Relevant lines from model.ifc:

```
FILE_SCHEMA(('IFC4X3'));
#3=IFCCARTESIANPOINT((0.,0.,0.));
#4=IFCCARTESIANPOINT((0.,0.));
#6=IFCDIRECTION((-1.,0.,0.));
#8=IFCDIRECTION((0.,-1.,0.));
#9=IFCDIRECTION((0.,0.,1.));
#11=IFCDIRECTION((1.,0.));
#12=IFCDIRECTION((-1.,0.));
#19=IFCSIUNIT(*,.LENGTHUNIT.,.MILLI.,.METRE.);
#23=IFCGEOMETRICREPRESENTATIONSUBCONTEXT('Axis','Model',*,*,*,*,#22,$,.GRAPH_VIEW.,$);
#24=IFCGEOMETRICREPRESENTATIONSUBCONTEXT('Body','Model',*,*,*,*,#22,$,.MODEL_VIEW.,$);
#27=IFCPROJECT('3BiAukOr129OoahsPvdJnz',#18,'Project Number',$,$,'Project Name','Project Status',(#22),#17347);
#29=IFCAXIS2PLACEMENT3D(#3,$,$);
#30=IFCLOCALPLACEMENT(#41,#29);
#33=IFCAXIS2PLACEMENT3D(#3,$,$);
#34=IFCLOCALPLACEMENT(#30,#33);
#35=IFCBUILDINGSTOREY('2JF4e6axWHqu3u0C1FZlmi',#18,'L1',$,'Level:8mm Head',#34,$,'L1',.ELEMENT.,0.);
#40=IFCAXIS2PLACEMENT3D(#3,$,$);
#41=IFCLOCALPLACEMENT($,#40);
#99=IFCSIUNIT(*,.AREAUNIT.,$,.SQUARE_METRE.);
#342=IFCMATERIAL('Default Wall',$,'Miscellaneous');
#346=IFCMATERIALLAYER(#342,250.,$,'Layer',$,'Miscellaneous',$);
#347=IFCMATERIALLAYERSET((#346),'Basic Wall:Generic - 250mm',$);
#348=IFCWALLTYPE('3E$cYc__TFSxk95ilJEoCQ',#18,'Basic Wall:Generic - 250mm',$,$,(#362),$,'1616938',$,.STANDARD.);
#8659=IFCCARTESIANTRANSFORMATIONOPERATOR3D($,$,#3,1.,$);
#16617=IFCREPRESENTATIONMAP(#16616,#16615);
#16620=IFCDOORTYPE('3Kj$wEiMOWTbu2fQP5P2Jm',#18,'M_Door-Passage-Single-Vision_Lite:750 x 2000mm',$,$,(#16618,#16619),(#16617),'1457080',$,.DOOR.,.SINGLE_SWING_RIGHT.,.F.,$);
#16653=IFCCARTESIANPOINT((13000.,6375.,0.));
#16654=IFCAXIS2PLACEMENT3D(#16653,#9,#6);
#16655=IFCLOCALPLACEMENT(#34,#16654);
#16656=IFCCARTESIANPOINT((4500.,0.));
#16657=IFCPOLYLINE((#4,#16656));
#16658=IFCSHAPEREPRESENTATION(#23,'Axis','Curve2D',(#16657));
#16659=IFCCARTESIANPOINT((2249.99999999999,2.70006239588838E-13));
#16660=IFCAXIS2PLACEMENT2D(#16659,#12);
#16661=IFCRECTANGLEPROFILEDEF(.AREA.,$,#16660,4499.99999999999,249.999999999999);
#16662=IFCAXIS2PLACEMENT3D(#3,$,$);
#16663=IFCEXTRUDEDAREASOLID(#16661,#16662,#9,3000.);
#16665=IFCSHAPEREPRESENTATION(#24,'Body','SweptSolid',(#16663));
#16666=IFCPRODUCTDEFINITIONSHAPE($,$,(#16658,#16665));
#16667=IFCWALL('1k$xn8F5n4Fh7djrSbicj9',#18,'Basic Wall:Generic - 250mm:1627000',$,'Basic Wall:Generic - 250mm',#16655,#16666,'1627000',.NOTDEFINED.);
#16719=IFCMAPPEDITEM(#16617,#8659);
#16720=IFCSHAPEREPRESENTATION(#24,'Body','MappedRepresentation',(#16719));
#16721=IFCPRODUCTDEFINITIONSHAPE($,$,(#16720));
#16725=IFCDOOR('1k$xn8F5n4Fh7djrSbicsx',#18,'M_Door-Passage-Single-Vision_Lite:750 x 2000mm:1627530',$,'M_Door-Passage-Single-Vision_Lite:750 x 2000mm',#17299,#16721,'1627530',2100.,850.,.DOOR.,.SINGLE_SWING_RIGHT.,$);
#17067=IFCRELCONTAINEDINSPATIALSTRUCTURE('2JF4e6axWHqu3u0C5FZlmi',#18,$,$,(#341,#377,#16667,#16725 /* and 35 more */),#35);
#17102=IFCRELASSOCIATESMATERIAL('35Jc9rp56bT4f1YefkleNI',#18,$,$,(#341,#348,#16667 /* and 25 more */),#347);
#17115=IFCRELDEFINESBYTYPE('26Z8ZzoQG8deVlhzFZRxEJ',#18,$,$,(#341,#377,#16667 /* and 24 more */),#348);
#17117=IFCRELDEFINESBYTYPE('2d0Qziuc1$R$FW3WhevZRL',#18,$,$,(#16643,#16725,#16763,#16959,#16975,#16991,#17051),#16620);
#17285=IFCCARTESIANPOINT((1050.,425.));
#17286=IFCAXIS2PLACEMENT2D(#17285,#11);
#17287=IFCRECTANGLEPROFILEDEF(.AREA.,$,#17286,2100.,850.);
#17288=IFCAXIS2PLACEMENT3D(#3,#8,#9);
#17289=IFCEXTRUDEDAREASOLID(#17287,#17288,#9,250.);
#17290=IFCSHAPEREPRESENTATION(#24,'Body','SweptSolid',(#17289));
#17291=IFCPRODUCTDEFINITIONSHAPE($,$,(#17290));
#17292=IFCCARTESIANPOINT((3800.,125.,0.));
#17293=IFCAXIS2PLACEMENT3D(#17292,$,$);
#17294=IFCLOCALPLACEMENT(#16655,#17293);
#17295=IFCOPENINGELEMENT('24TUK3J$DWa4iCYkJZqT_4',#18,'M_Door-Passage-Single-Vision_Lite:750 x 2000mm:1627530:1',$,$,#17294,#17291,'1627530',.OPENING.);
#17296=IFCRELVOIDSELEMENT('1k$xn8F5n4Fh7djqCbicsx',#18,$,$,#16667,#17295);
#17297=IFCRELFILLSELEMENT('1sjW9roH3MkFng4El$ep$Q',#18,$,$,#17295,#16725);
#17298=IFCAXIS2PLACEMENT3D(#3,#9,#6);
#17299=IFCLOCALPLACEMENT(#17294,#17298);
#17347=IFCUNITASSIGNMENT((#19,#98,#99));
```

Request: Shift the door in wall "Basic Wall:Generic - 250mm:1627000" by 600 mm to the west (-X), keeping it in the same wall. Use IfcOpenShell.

```python
import ifcopenshell
import ifcopenshell.api.geometry
import ifcopenshell.util.placement

model = ifcopenshell.open("model.ifc")

door = model.by_id(16725)
opening = door.FillsVoids[0].RelatingOpeningElement
wall = opening.VoidsElements[0].RelatingBuildingElement

wall_matrix = ifcopenshell.util.placement.get_local_placement(wall.ObjectPlacement)
shift = wall_matrix[:3, 0] * 600.0
before = ifcopenshell.util.placement.get_local_placement(door.ObjectPlacement)[:3, 3].copy()

# The door is placed relative to its opening, so it follows when the opening moves.
matrix = ifcopenshell.util.placement.get_local_placement(opening.ObjectPlacement)
matrix[:3, 3] += shift
ifcopenshell.api.geometry.edit_object_placement(
    model, product=opening, matrix=matrix, is_si=False, should_transform_children=True
)

after = ifcopenshell.util.placement.get_local_placement(door.ObjectPlacement)[:3, 3]
print("door moved by", (after - before).round(3) + 0.0)

model.write("model_rev.ifc")
```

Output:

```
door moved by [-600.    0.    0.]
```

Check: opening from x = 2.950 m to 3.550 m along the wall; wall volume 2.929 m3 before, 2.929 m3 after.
